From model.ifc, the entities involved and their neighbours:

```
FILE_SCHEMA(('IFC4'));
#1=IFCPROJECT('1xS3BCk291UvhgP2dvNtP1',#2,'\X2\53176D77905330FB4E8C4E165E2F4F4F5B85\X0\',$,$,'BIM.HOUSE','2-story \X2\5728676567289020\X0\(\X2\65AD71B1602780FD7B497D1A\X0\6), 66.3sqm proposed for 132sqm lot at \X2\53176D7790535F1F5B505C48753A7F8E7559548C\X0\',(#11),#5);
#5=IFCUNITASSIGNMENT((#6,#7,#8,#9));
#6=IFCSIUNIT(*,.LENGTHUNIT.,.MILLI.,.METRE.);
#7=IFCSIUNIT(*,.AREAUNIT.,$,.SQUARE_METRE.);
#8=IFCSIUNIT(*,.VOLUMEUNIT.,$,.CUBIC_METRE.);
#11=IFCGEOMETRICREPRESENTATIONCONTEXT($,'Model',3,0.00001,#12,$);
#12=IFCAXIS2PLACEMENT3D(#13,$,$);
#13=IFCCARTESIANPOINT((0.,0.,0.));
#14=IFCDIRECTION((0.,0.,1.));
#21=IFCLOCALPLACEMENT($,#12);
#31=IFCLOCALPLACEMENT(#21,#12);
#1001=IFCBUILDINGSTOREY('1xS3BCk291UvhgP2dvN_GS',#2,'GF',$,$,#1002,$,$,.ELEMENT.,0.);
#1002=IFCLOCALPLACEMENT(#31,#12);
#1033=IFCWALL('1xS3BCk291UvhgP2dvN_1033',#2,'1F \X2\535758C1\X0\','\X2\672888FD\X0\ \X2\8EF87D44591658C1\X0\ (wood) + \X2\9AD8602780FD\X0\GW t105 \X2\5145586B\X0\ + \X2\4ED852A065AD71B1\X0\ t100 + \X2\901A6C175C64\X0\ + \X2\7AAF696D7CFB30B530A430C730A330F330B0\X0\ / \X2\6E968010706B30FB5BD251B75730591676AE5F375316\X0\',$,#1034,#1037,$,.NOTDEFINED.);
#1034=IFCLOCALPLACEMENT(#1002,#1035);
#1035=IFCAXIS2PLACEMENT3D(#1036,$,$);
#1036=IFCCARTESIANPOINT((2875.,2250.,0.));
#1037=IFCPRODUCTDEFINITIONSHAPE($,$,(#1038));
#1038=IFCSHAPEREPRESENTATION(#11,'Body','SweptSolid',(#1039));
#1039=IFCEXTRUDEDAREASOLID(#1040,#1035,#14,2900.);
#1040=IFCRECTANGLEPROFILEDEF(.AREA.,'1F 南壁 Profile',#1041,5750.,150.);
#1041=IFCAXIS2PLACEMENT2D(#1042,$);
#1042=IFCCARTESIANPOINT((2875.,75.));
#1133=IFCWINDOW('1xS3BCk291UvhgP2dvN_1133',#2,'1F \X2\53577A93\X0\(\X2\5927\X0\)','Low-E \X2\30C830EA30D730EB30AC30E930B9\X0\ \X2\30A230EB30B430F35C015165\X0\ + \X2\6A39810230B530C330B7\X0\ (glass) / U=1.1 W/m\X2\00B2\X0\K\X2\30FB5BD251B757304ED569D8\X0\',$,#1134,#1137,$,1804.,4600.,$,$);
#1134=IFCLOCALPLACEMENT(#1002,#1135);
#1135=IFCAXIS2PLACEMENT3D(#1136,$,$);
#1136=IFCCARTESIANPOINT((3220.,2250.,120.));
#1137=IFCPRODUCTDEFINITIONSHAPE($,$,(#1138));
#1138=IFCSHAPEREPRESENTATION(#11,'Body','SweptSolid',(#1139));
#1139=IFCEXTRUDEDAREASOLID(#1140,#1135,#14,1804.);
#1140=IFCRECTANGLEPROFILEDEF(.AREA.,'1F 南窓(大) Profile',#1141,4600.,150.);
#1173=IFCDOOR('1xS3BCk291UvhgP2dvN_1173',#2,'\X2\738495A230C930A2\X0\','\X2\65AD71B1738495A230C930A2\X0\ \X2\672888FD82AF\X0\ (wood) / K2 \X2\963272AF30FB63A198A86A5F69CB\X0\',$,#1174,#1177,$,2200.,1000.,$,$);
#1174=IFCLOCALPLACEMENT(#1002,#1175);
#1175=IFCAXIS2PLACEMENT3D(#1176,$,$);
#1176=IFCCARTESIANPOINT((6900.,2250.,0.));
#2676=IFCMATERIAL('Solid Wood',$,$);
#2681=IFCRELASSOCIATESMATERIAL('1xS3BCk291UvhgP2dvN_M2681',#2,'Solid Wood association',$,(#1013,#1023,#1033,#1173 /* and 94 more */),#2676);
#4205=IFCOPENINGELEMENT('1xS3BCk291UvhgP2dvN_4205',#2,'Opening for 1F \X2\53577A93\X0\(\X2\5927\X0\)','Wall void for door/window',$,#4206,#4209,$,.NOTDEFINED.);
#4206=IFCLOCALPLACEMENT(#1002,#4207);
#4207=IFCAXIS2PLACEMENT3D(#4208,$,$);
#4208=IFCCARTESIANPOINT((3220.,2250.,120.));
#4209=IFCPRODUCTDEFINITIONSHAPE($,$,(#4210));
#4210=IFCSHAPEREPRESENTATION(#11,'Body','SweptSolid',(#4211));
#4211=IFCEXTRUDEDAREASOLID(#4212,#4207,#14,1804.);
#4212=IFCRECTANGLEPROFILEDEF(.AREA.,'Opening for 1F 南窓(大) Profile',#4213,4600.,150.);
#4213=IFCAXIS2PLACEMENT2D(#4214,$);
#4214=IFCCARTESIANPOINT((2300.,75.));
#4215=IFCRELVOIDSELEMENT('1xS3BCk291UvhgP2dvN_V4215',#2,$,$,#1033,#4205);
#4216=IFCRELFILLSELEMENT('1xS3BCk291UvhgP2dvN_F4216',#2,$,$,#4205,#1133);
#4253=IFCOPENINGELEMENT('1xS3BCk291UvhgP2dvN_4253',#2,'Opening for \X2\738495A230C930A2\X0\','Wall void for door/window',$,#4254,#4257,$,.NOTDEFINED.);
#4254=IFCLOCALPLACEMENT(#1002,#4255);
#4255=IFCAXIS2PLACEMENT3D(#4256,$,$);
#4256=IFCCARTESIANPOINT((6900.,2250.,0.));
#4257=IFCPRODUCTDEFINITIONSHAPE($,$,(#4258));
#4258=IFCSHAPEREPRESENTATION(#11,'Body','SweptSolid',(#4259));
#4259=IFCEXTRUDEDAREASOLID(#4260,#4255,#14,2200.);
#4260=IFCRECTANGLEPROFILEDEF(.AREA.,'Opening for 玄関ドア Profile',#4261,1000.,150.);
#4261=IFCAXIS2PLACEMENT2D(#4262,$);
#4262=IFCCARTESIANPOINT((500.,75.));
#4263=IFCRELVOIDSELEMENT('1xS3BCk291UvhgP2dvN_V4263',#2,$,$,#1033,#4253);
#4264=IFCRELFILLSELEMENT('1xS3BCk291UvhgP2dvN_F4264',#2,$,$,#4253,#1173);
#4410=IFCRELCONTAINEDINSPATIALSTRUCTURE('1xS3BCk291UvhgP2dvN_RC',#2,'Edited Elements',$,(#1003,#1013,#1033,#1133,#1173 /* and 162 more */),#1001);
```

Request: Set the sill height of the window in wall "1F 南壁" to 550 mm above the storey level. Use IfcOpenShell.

```python
import numpy as np
import ifcopenshell
import ifcopenshell.api.geometry
import ifcopenshell.geom
import ifcopenshell.util.element
import ifcopenshell.util.placement
import ifcopenshell.util.shape
import ifcopenshell.util.unit

model = ifcopenshell.open("model.ifc")
unit_scale = ifcopenshell.util.unit.calculate_unit_scale(model)

window = model.by_guid("1xS3BCk291UvhgP2dvN_1133")
opening = window.FillsVoids[0].RelatingOpeningElement
storey = ifcopenshell.util.element.get_container(window, ifc_class="IfcBuildingStorey")
level = ifcopenshell.util.placement.get_local_placement(storey.ObjectPlacement)[2, 3]

# The opening's origin need not be at the sill, so measure its lowest point.
shape = ifcopenshell.geom.create_shape(ifcopenshell.geom.settings(), opening)
bottom = ifcopenshell.util.shape.get_shape_bottom_elevation(shape, shape.geometry) / unit_scale
dz = level + 0.55 / unit_scale - bottom

shift = np.array([0.0, 0.0, dz])
# The window is not placed relative to its opening, so move both.
for product in (opening, window):
    matrix = ifcopenshell.util.placement.get_local_placement(product.ObjectPlacement)
    matrix[:3, 3] += shift
    ifcopenshell.api.geometry.edit_object_placement(model, product=product, matrix=matrix, is_si=False)

print(f"moved by {dz * unit_scale:+.3f} m")

model.write("model-out.ifc")
```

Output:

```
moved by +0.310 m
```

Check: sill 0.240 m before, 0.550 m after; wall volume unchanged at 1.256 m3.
